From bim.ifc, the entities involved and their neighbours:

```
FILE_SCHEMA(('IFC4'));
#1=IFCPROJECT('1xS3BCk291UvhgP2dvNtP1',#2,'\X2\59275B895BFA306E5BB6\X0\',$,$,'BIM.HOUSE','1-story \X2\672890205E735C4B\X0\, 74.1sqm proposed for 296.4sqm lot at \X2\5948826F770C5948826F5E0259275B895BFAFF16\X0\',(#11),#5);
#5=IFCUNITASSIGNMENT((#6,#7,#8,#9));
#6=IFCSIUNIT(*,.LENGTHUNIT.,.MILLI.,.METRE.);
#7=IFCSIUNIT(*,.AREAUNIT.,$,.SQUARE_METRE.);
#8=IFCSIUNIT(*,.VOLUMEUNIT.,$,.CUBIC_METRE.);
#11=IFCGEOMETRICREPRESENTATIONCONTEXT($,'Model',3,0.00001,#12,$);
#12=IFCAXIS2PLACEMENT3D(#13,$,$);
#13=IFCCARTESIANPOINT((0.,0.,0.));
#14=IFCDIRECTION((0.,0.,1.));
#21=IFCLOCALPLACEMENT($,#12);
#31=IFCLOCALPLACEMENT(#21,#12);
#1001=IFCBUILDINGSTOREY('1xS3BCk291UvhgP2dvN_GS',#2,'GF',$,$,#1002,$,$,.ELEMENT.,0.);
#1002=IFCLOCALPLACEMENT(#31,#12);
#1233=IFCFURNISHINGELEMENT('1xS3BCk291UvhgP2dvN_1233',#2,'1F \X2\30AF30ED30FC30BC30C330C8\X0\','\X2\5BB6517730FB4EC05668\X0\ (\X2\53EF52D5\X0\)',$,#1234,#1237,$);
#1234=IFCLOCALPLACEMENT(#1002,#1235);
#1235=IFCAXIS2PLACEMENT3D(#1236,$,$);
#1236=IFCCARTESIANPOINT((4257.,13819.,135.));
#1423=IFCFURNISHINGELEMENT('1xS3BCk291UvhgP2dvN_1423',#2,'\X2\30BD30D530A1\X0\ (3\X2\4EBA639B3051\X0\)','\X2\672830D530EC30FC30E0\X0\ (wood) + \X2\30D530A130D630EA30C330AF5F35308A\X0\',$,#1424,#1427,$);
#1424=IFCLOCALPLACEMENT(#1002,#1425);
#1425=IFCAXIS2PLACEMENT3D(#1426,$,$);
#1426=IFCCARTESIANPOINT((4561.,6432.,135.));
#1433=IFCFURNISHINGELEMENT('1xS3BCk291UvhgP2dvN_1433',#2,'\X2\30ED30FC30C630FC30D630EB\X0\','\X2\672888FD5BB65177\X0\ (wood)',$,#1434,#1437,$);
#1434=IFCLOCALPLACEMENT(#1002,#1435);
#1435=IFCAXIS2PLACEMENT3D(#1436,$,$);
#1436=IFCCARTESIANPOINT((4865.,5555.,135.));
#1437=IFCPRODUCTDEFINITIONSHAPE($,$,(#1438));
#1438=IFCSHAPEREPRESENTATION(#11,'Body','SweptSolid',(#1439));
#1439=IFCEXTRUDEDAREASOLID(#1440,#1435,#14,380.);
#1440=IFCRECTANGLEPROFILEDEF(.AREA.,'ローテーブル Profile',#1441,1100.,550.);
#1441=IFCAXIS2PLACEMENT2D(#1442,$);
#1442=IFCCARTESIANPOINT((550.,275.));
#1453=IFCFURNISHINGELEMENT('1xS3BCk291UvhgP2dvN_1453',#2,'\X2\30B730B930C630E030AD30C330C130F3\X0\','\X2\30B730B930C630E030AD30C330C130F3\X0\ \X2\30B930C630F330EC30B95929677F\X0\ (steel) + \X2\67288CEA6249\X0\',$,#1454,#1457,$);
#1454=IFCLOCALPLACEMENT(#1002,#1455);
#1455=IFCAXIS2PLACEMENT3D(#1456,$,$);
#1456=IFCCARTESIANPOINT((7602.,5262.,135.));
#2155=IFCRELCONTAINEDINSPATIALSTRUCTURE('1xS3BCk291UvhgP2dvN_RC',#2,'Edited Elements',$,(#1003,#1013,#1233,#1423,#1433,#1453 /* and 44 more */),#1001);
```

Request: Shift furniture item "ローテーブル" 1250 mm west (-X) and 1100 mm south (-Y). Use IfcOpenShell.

```python
import ifcopenshell
import ifcopenshell.api.geometry
import ifcopenshell.util.placement

model = ifcopenshell.open("bim.ifc")

item = model.by_id(1433)
matrix = ifcopenshell.util.placement.get_local_placement(item.ObjectPlacement)
matrix[0, 3] -= 1250.0
matrix[1, 3] -= 1100.0
ifcopenshell.api.geometry.edit_object_placement(model, product=item, matrix=matrix, is_si=False)

print(ifcopenshell.util.placement.get_local_placement(item.ObjectPlacement).round(3) + 0.0)

model.write("bim_edited.ifc")
```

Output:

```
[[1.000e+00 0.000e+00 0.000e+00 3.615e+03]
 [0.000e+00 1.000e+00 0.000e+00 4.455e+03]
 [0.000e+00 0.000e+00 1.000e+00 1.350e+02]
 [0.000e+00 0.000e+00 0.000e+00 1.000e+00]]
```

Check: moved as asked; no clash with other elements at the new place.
